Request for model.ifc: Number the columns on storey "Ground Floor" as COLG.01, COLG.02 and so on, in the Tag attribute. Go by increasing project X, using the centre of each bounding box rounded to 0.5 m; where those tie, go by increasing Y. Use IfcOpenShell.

First a look at what the model holds.

```python
import ifcopenshell
import ifcopenshell.util.element
import ifcopenshell.util.placement

model = ifcopenshell.open("model.ifc")
print(model.schema)
storey = next(s for s in model.by_type("IfcBuildingStorey") if s.Name == "Ground Floor")
columns = [e for e in ifcopenshell.util.element.get_decomposition(storey) if e.is_a("IfcColumn")]
for e in sorted(columns, key=lambda e: e.id()):
    origin = ifcopenshell.util.placement.get_local_placement(e.ObjectPlacement)[:3, 3]
    print(e.id(), e.Tag, e.Name, origin.round(2) + 0.0, sep=" | ")
```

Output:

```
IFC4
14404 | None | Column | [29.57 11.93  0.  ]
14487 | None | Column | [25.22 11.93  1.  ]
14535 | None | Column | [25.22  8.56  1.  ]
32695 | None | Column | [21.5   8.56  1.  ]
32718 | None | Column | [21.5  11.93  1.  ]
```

```python
import ifcopenshell
import ifcopenshell.geom
import ifcopenshell.util.element
import ifcopenshell.util.shape

model = ifcopenshell.open("model.ifc")
settings = ifcopenshell.geom.settings()
settings.set("use-world-coords", True)


def centre(element):
    shape = ifcopenshell.geom.create_shape(settings, element)
    return ifcopenshell.util.shape.get_bbox_centroid(shape.geometry)


storey = next(s for s in model.by_type("IfcBuildingStorey") if s.Name == "Ground Floor")
columns = [e for e in ifcopenshell.util.element.get_decomposition(storey) if e.is_a("IfcColumn")]

# Insertion points can sit at a corner or the storey origin, so sort by the geometry (in metres).
centres = {e: centre(e) for e in columns}
columns.sort(key=lambda e: (round(centres[e][0] / 0.5), centres[e][1]))

for i, e in enumerate(columns, start=1):
    number = f"COLG.{i:02d}"
    e.Tag = number
    print(e.id(), number)

model.write("model_updated.ifc")
```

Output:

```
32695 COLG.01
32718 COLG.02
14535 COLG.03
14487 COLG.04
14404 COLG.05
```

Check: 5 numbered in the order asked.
